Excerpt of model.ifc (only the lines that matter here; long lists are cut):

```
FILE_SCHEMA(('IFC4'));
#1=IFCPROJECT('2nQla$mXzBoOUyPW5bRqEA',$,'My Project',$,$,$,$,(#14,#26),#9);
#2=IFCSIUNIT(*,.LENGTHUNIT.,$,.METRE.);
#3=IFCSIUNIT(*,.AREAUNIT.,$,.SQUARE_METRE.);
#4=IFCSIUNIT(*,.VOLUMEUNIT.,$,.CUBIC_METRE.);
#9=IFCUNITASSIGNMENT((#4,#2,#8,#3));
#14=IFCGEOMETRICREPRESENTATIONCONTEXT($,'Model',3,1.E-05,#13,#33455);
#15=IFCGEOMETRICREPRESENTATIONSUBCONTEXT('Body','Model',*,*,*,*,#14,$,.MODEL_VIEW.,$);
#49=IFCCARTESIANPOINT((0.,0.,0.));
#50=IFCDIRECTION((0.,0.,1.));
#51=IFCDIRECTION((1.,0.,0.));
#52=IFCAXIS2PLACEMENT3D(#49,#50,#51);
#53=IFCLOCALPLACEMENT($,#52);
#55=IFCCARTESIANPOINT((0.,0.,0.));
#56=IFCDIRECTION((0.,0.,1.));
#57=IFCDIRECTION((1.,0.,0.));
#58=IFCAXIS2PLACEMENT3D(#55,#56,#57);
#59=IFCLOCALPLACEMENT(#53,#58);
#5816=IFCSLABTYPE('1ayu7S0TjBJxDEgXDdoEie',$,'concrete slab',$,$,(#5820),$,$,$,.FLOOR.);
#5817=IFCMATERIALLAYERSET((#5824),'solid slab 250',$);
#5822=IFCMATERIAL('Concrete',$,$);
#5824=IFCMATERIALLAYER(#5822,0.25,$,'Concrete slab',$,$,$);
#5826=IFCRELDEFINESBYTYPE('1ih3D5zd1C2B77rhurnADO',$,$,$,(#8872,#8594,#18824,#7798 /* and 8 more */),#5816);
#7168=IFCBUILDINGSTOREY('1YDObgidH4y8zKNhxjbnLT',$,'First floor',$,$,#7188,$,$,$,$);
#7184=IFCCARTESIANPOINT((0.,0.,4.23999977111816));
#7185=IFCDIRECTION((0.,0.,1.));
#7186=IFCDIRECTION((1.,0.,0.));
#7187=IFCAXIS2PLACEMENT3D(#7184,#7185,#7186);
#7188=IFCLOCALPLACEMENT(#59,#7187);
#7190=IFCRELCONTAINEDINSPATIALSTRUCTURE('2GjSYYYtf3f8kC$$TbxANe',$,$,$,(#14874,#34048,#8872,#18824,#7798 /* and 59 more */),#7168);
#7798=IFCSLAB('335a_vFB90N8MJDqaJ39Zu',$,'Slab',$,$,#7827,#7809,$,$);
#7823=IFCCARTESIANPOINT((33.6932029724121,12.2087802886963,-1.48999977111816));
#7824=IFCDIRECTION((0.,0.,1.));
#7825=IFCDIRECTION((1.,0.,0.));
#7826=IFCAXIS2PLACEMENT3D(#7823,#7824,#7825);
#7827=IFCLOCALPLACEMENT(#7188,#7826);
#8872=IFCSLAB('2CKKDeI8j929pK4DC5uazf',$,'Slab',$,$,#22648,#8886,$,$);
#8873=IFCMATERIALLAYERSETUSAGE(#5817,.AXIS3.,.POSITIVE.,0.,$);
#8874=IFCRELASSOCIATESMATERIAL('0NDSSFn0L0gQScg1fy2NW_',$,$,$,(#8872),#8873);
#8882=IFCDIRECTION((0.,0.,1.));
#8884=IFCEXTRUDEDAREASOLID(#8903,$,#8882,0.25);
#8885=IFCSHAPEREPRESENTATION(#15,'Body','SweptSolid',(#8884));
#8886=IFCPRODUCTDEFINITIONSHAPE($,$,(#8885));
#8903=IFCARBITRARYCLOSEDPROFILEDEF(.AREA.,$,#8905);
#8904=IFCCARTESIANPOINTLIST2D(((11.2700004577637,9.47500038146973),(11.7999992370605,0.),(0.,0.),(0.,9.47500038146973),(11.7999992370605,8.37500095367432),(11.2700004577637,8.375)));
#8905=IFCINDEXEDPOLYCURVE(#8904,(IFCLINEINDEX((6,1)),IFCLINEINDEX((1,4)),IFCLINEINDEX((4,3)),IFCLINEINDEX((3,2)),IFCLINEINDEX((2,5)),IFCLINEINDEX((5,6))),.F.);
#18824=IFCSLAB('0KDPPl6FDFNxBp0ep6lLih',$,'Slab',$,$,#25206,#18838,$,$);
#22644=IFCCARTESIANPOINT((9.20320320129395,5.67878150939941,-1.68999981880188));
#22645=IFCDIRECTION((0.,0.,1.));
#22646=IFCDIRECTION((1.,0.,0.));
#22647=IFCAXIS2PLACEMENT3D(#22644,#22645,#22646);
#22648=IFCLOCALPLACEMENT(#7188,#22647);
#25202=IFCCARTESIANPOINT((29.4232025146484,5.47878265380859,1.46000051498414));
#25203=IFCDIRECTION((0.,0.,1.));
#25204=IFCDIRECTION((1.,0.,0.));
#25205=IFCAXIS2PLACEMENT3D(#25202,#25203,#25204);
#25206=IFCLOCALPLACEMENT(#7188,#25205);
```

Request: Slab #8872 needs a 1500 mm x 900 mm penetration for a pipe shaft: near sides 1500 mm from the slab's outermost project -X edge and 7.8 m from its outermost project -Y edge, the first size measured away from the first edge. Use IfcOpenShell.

```python
import numpy as np
import ifcopenshell
import ifcopenshell.api.feature
import ifcopenshell.api.geometry
import ifcopenshell.api.root
import ifcopenshell.geom
import ifcopenshell.util.placement
import ifcopenshell.util.representation
import ifcopenshell.util.shape
import ifcopenshell.util.unit

model = ifcopenshell.open("model.ifc")
unit_scale = ifcopenshell.util.unit.calculate_unit_scale(model)
settings = ifcopenshell.geom.settings()


def volume(element):
    """Net volume in cubic metres, openings subtracted."""
    shape = ifcopenshell.geom.create_shape(settings, element)
    return ifcopenshell.util.shape.get_volume(shape.geometry)


slab = model.by_id(8872)
before = volume(slab)

# Extent in the slab's own axes, in metres. The edges named are its -X and -Y sides.
slab_shape = ifcopenshell.geom.create_shape(settings, slab)
vertices = ifcopenshell.util.shape.get_vertices(slab_shape.geometry)
x_min, y_min, bottom = vertices.min(axis=0)
top = vertices[:, 2].max()

opening = ifcopenshell.api.root.create_entity(model, ifc_class="IfcOpeningElement", name="Pipe shaft opening", predefined_type="OPENING")
context = ifcopenshell.util.representation.get_context(model, "Model", "Body", "MODEL_VIEW")
width, depth = 1.5, 0.9
outline = [(0.0, 0.0), (width, 0.0), (width, depth), (0.0, depth), (0.0, 0.0)]
# Overshoot both faces by 50 mm so the cut is clean.
shape = ifcopenshell.api.geometry.add_slab_representation(
    model, context=context, depth=top - bottom + 0.1, polyline=outline
)
ifcopenshell.api.geometry.assign_representation(model, product=opening, representation=shape)

matrix = ifcopenshell.util.placement.get_local_placement(slab.ObjectPlacement)
matrix[:, 3] = matrix @ np.append(np.array([x_min + 1.5, y_min + 7.8, bottom - 0.05]) / unit_scale, 1.0)
ifcopenshell.api.geometry.edit_object_placement(model, product=opening, matrix=matrix, is_si=False)
ifcopenshell.api.feature.add_feature(model, feature=opening, element=slab)

after = volume(slab)

print(f"slab volume {before:.3f} -> {after:.3f} m3")

model.write("model_rev.ifc")
```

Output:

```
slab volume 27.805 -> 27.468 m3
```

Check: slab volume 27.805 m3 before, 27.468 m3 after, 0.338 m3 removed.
